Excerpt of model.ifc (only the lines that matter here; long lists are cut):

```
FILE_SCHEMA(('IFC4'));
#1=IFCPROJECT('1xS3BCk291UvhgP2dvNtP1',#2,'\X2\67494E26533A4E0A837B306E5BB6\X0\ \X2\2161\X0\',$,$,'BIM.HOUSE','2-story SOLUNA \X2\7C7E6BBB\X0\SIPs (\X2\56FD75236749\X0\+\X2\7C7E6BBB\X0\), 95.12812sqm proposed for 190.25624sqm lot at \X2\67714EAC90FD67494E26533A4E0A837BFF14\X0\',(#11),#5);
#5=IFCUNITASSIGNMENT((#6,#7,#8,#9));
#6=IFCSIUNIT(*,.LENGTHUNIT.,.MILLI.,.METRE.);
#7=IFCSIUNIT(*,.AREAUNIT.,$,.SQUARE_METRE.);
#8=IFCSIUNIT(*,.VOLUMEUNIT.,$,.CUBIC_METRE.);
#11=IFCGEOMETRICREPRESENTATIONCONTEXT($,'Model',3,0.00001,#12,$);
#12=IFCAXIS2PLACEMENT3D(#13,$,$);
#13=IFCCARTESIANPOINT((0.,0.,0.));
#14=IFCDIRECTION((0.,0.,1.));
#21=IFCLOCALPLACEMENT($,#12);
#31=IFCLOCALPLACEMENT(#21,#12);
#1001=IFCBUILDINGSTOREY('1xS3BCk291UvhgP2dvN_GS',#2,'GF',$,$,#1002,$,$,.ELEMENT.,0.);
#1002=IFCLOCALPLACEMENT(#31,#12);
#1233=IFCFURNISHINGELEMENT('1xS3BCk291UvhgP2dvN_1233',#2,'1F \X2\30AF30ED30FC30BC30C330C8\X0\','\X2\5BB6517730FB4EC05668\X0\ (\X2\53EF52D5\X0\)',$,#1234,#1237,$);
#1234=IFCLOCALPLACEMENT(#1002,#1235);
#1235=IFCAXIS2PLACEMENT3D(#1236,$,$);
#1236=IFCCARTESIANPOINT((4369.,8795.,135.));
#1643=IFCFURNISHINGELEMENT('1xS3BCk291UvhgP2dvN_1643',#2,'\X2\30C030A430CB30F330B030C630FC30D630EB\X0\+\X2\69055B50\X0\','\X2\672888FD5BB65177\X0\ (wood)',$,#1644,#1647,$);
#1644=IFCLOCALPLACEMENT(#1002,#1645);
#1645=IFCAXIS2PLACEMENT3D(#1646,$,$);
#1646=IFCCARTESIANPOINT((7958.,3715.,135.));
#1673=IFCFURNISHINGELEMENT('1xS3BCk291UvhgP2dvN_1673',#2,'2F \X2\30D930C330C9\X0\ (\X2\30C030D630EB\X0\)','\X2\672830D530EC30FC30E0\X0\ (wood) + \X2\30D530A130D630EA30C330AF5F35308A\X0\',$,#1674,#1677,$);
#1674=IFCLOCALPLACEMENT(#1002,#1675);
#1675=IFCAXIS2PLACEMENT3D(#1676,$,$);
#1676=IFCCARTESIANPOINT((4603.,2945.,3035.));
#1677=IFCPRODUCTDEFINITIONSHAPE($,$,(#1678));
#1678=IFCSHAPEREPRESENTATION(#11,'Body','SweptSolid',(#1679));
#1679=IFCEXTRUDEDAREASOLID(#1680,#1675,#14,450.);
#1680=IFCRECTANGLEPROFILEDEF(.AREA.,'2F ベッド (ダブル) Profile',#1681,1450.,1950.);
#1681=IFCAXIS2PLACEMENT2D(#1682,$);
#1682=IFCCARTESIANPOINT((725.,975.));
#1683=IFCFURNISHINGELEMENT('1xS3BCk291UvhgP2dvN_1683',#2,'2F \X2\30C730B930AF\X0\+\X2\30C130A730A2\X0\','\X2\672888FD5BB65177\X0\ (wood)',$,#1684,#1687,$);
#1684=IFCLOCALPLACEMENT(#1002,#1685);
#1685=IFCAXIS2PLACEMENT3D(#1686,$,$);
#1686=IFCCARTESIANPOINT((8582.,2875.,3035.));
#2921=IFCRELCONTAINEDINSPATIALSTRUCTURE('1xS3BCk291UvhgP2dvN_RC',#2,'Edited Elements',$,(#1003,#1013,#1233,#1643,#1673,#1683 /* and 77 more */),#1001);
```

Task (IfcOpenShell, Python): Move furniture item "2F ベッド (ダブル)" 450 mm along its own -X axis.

```python
import ifcopenshell
import ifcopenshell.api.geometry
import ifcopenshell.util.placement

model = ifcopenshell.open("model.ifc")

item = model.by_guid("1xS3BCk291UvhgP2dvN_1673")
matrix = ifcopenshell.util.placement.get_local_placement(item.ObjectPlacement)
matrix[:3, 3] -= matrix[:3, 0] * 450.0
ifcopenshell.api.geometry.edit_object_placement(model, product=item, matrix=matrix, is_si=False)

print(ifcopenshell.util.placement.get_local_placement(item.ObjectPlacement).round(3) + 0.0)

model.write("model_updated.ifc")
```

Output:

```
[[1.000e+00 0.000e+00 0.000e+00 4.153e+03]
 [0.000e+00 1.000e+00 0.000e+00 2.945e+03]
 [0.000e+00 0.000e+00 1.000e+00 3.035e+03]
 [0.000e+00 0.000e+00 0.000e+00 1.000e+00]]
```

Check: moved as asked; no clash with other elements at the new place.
